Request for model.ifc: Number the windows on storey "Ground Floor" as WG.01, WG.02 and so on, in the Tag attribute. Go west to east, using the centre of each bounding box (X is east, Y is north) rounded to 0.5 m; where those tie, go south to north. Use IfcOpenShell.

First a look at what the model holds.

```python
import ifcopenshell
import ifcopenshell.util.element
import ifcopenshell.util.placement

model = ifcopenshell.open("model.ifc")
print(model.schema)
storey = next(s for s in model.by_type("IfcBuildingStorey") if s.Name == "Ground Floor")
windows = [e for e in ifcopenshell.util.element.get_decomposition(storey) if e.is_a("IfcWindow")]
for e in sorted(windows, key=lambda e: e.id()):
    origin = ifcopenshell.util.placement.get_local_placement(e.ObjectPlacement)[:3, 3]
    print(e.id(), e.Tag, e.Name, origin.round(2) + 0.0, sep=" | ")
```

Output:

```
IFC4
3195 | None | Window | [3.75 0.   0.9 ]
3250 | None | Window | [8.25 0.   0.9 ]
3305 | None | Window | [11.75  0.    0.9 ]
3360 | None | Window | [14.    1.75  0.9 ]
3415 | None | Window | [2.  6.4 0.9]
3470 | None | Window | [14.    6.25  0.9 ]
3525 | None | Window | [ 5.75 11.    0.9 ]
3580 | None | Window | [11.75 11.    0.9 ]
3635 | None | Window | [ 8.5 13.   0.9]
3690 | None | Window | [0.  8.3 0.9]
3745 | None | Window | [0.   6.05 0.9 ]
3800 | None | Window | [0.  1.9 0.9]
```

```python
import ifcopenshell
import ifcopenshell.geom
import ifcopenshell.util.element
import ifcopenshell.util.shape

model = ifcopenshell.open("model.ifc")
settings = ifcopenshell.geom.settings()
settings.set("use-world-coords", True)


def centre(element):
    shape = ifcopenshell.geom.create_shape(settings, element)
    return ifcopenshell.util.shape.get_bbox_centroid(shape.geometry)


storey = next(s for s in model.by_type("IfcBuildingStorey") if s.Name == "Ground Floor")
windows = [e for e in ifcopenshell.util.element.get_decomposition(storey) if e.is_a("IfcWindow")]

# Insertion points can sit at a corner or the storey origin, so sort by the geometry (in metres).
centres = {e: centre(e) for e in windows}
windows.sort(key=lambda e: (round(centres[e][0] / 0.5), centres[e][1]))

for i, e in enumerate(windows, start=1):
    number = f"WG.{i:02d}"
    e.Tag = number
    print(e.id(), number)

model.write("model_rev.ifc")
```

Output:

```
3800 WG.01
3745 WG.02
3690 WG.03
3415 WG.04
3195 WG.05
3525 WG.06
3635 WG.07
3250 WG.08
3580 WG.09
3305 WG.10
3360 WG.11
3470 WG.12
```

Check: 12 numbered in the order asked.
